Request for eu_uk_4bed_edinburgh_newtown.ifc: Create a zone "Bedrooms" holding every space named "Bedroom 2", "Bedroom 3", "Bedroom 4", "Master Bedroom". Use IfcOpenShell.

First a look at what the model holds.

```python
import ifcopenshell

model = ifcopenshell.open("eu_uk_4bed_edinburgh_newtown.ifc")
print(model.schema)
seen = {}
for space in model.by_type("IfcSpace"):
    seen[space.LongName] = seen.get(space.LongName, 0) + 1
for name, count in sorted(seen.items(), key=str):
    print(count, "x", name)
print("zones:", [z.Name for z in model.by_type("IfcZone")][:20])
```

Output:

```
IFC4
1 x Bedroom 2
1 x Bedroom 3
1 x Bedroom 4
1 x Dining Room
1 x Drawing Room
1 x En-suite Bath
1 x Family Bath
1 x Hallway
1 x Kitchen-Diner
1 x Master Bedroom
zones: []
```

```python
import ifcopenshell
import ifcopenshell.api.group
import ifcopenshell.api.root

model = ifcopenshell.open("eu_uk_4bed_edinburgh_newtown.ifc")

names = {"Bedroom 2", "Bedroom 3", "Bedroom 4", "Master Bedroom"}
spaces = [s for s in model.by_type("IfcSpace") if s.LongName in names]

zone = ifcopenshell.api.root.create_entity(model, ifc_class="IfcZone", name="Bedrooms")
ifcopenshell.api.group.assign_group(model, products=spaces, group=zone)
print(len(spaces), "spaces in", zone.Name)

model.write("eu_uk_4bed_edinburgh_newtown-out.ifc")
```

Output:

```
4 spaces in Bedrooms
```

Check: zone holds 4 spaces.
